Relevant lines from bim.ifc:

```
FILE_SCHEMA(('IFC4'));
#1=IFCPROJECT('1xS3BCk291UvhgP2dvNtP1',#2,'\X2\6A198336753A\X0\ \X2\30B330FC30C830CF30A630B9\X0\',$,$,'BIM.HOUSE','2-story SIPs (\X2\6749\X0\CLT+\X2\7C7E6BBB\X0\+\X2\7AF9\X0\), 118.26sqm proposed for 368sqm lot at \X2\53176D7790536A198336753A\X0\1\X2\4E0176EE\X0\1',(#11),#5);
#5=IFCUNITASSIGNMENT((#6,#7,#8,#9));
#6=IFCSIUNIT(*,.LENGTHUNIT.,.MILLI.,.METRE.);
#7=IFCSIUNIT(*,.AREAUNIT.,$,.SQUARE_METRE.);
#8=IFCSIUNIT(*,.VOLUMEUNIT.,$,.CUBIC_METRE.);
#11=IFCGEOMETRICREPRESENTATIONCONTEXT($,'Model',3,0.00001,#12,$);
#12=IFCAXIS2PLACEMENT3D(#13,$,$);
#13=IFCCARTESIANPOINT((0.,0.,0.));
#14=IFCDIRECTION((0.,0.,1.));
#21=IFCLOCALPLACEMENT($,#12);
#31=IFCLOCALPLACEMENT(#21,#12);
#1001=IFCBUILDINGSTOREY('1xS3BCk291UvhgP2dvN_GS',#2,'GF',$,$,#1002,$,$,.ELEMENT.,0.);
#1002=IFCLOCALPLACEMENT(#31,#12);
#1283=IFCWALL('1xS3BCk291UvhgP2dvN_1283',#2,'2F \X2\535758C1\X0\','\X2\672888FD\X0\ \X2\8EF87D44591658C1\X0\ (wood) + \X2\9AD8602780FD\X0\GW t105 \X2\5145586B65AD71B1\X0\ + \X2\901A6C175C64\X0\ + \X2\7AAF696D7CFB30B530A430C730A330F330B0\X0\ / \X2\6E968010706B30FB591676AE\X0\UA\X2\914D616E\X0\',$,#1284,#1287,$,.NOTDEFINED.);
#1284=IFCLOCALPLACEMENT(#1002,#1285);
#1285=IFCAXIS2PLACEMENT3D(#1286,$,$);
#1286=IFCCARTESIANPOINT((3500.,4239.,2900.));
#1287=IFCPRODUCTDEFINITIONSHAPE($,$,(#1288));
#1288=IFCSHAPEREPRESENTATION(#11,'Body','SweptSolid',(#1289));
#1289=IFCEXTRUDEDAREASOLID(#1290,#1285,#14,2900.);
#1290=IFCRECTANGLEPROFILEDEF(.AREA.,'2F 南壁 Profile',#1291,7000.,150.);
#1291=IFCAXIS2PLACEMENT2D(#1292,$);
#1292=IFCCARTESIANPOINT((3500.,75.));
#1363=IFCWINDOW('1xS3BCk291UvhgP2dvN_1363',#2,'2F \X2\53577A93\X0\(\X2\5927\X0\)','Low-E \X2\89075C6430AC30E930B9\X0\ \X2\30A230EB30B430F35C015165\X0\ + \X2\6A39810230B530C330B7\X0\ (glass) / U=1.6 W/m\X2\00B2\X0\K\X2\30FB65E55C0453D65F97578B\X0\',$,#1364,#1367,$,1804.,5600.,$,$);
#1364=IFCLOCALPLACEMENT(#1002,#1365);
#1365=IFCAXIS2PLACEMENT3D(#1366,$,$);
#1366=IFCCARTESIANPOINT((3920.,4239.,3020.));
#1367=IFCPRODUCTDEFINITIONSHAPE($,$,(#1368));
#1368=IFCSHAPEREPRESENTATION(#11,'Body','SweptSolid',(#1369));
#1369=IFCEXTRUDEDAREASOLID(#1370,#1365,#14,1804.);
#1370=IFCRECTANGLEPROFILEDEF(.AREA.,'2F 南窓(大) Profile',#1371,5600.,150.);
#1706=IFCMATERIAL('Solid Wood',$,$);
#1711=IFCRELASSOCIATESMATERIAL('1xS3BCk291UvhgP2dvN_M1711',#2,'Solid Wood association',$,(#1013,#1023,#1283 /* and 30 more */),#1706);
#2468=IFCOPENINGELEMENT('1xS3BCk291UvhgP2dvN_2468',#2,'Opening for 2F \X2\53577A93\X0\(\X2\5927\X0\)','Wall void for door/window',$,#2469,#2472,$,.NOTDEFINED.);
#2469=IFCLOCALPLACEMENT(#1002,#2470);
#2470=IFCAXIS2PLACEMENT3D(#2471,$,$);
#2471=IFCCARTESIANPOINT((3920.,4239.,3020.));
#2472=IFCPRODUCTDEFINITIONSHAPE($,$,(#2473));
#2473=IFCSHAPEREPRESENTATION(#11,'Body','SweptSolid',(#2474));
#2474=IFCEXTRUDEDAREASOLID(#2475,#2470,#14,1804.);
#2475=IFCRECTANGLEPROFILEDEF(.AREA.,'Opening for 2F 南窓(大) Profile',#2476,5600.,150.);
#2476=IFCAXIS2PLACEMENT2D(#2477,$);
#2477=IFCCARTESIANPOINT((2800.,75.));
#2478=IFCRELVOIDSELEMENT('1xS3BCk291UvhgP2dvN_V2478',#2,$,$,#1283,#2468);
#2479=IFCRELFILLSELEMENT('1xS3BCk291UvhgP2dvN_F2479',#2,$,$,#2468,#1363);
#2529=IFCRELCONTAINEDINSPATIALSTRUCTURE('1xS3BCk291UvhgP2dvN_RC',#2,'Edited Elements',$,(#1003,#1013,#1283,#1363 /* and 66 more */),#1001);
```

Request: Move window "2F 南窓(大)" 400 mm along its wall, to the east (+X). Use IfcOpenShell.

```python
import ifcopenshell
import ifcopenshell.api.geometry
import ifcopenshell.util.placement
import ifcopenshell.util.unit

model = ifcopenshell.open("bim.ifc")
unit_scale = ifcopenshell.util.unit.calculate_unit_scale(model)

window = model.by_guid("1xS3BCk291UvhgP2dvN_1363")
opening = window.FillsVoids[0].RelatingOpeningElement
wall = opening.VoidsElements[0].RelatingBuildingElement

wall_matrix = ifcopenshell.util.placement.get_local_placement(wall.ObjectPlacement)
shift = wall_matrix[:3, 0] * 0.4 / unit_scale
before = ifcopenshell.util.placement.get_local_placement(window.ObjectPlacement)[:3, 3].copy()

# The window is not placed relative to its opening, so move both.
for product in (opening, window):
    matrix = ifcopenshell.util.placement.get_local_placement(product.ObjectPlacement)
    matrix[:3, 3] += shift
    ifcopenshell.api.geometry.edit_object_placement(model, product=product, matrix=matrix, is_si=False)

after = ifcopenshell.util.placement.get_local_placement(window.ObjectPlacement)[:3, 3]
print("window moved by", (after - before).round(3) + 0.0)

model.write("bim_v2.ifc")
```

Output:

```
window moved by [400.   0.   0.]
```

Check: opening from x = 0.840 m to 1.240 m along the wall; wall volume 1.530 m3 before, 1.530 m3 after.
